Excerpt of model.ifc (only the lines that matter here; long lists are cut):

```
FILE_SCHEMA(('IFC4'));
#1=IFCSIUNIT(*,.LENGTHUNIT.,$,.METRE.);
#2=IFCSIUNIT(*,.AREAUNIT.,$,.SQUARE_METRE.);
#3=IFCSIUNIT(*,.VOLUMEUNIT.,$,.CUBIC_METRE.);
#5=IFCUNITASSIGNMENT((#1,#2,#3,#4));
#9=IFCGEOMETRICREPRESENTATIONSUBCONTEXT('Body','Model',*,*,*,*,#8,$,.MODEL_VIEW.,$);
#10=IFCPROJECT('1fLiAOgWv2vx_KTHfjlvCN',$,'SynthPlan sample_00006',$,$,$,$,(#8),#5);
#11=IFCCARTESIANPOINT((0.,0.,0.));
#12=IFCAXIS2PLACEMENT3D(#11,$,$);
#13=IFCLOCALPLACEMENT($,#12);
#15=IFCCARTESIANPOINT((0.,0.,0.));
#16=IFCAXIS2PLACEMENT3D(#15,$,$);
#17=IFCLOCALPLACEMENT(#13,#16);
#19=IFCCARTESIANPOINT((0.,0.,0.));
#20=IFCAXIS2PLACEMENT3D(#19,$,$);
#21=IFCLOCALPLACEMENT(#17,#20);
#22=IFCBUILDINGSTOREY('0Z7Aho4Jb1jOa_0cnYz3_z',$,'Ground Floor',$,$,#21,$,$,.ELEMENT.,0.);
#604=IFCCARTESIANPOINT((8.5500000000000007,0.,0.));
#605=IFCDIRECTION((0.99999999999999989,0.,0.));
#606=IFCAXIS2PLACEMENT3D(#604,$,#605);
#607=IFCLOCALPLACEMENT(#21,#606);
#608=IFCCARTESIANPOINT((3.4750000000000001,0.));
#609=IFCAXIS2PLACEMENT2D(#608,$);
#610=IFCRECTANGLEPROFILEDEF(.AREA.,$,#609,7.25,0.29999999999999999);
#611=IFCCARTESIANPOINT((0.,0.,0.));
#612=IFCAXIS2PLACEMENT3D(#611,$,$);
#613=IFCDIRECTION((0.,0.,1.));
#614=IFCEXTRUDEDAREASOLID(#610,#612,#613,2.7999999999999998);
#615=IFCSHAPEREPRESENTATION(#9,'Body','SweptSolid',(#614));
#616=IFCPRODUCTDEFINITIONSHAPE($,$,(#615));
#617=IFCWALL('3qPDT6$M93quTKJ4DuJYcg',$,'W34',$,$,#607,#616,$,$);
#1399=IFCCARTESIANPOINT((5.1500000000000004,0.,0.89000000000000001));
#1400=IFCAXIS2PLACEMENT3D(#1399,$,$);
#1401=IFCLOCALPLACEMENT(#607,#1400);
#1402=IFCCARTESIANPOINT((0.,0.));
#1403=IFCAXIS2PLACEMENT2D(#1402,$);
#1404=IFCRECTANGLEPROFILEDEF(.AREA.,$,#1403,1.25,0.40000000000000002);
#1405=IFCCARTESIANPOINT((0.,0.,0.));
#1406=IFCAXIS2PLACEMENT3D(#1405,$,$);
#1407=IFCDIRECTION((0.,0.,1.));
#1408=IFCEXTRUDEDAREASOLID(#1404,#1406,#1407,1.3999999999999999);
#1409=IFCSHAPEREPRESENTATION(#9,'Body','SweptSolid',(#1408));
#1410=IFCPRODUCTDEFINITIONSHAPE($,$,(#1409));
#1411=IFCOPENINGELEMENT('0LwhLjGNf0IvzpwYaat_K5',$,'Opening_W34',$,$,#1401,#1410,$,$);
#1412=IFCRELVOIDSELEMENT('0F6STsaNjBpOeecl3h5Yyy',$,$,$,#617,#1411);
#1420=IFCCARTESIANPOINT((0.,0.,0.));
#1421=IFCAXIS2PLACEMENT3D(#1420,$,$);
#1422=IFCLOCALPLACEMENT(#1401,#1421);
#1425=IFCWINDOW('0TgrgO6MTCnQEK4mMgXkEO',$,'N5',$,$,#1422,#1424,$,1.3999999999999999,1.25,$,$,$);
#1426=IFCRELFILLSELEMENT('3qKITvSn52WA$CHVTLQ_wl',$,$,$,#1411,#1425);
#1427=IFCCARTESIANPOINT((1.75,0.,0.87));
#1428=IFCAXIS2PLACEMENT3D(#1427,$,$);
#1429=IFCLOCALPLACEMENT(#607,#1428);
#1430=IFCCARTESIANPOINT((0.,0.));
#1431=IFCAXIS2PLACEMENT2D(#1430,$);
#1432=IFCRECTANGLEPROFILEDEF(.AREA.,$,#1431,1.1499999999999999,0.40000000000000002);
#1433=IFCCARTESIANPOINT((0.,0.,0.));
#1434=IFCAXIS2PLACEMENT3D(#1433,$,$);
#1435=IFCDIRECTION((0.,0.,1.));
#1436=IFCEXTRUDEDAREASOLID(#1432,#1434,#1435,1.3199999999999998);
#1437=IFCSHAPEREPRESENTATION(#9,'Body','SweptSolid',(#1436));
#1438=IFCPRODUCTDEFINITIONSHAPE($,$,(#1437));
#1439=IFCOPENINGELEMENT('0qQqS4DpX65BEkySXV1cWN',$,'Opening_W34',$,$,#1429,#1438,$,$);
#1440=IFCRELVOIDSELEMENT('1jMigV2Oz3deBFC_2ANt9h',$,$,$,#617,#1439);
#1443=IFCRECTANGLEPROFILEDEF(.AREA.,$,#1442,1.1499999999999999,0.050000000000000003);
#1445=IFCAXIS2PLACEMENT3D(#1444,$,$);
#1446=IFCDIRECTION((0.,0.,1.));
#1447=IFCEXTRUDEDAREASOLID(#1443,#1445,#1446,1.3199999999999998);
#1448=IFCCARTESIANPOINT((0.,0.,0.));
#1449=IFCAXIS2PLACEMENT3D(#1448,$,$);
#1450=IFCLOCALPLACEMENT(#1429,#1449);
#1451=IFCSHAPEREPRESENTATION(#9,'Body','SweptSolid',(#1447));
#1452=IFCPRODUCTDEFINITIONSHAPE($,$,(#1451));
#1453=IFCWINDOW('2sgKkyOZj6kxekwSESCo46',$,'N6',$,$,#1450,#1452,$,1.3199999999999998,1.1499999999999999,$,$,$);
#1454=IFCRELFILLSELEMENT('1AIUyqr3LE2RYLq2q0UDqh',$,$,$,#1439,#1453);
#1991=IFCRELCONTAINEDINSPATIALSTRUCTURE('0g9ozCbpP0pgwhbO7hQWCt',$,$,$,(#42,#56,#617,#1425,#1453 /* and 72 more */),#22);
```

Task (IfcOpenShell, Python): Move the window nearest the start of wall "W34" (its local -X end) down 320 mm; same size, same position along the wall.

```python
import numpy as np
import ifcopenshell
import ifcopenshell.api.geometry
import ifcopenshell.util.placement
import ifcopenshell.util.unit

model = ifcopenshell.open("model.ifc")
unit_scale = ifcopenshell.util.unit.calculate_unit_scale(model)

window = model.by_guid("2sgKkyOZj6kxekwSESCo46")
opening = window.FillsVoids[0].RelatingOpeningElement
dz = -0.32 / unit_scale

shift = np.array([0.0, 0.0, dz])
# The window is placed relative to its opening, so it follows when the opening moves.
matrix = ifcopenshell.util.placement.get_local_placement(opening.ObjectPlacement)
matrix[:3, 3] += shift
ifcopenshell.api.geometry.edit_object_placement(
    model, product=opening, matrix=matrix, is_si=False, should_transform_children=True
)

print(f"moved by {dz * unit_scale:+.3f} m")

model.write("model_v2.ifc")
```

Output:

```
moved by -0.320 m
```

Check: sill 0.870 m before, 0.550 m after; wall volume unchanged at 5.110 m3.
